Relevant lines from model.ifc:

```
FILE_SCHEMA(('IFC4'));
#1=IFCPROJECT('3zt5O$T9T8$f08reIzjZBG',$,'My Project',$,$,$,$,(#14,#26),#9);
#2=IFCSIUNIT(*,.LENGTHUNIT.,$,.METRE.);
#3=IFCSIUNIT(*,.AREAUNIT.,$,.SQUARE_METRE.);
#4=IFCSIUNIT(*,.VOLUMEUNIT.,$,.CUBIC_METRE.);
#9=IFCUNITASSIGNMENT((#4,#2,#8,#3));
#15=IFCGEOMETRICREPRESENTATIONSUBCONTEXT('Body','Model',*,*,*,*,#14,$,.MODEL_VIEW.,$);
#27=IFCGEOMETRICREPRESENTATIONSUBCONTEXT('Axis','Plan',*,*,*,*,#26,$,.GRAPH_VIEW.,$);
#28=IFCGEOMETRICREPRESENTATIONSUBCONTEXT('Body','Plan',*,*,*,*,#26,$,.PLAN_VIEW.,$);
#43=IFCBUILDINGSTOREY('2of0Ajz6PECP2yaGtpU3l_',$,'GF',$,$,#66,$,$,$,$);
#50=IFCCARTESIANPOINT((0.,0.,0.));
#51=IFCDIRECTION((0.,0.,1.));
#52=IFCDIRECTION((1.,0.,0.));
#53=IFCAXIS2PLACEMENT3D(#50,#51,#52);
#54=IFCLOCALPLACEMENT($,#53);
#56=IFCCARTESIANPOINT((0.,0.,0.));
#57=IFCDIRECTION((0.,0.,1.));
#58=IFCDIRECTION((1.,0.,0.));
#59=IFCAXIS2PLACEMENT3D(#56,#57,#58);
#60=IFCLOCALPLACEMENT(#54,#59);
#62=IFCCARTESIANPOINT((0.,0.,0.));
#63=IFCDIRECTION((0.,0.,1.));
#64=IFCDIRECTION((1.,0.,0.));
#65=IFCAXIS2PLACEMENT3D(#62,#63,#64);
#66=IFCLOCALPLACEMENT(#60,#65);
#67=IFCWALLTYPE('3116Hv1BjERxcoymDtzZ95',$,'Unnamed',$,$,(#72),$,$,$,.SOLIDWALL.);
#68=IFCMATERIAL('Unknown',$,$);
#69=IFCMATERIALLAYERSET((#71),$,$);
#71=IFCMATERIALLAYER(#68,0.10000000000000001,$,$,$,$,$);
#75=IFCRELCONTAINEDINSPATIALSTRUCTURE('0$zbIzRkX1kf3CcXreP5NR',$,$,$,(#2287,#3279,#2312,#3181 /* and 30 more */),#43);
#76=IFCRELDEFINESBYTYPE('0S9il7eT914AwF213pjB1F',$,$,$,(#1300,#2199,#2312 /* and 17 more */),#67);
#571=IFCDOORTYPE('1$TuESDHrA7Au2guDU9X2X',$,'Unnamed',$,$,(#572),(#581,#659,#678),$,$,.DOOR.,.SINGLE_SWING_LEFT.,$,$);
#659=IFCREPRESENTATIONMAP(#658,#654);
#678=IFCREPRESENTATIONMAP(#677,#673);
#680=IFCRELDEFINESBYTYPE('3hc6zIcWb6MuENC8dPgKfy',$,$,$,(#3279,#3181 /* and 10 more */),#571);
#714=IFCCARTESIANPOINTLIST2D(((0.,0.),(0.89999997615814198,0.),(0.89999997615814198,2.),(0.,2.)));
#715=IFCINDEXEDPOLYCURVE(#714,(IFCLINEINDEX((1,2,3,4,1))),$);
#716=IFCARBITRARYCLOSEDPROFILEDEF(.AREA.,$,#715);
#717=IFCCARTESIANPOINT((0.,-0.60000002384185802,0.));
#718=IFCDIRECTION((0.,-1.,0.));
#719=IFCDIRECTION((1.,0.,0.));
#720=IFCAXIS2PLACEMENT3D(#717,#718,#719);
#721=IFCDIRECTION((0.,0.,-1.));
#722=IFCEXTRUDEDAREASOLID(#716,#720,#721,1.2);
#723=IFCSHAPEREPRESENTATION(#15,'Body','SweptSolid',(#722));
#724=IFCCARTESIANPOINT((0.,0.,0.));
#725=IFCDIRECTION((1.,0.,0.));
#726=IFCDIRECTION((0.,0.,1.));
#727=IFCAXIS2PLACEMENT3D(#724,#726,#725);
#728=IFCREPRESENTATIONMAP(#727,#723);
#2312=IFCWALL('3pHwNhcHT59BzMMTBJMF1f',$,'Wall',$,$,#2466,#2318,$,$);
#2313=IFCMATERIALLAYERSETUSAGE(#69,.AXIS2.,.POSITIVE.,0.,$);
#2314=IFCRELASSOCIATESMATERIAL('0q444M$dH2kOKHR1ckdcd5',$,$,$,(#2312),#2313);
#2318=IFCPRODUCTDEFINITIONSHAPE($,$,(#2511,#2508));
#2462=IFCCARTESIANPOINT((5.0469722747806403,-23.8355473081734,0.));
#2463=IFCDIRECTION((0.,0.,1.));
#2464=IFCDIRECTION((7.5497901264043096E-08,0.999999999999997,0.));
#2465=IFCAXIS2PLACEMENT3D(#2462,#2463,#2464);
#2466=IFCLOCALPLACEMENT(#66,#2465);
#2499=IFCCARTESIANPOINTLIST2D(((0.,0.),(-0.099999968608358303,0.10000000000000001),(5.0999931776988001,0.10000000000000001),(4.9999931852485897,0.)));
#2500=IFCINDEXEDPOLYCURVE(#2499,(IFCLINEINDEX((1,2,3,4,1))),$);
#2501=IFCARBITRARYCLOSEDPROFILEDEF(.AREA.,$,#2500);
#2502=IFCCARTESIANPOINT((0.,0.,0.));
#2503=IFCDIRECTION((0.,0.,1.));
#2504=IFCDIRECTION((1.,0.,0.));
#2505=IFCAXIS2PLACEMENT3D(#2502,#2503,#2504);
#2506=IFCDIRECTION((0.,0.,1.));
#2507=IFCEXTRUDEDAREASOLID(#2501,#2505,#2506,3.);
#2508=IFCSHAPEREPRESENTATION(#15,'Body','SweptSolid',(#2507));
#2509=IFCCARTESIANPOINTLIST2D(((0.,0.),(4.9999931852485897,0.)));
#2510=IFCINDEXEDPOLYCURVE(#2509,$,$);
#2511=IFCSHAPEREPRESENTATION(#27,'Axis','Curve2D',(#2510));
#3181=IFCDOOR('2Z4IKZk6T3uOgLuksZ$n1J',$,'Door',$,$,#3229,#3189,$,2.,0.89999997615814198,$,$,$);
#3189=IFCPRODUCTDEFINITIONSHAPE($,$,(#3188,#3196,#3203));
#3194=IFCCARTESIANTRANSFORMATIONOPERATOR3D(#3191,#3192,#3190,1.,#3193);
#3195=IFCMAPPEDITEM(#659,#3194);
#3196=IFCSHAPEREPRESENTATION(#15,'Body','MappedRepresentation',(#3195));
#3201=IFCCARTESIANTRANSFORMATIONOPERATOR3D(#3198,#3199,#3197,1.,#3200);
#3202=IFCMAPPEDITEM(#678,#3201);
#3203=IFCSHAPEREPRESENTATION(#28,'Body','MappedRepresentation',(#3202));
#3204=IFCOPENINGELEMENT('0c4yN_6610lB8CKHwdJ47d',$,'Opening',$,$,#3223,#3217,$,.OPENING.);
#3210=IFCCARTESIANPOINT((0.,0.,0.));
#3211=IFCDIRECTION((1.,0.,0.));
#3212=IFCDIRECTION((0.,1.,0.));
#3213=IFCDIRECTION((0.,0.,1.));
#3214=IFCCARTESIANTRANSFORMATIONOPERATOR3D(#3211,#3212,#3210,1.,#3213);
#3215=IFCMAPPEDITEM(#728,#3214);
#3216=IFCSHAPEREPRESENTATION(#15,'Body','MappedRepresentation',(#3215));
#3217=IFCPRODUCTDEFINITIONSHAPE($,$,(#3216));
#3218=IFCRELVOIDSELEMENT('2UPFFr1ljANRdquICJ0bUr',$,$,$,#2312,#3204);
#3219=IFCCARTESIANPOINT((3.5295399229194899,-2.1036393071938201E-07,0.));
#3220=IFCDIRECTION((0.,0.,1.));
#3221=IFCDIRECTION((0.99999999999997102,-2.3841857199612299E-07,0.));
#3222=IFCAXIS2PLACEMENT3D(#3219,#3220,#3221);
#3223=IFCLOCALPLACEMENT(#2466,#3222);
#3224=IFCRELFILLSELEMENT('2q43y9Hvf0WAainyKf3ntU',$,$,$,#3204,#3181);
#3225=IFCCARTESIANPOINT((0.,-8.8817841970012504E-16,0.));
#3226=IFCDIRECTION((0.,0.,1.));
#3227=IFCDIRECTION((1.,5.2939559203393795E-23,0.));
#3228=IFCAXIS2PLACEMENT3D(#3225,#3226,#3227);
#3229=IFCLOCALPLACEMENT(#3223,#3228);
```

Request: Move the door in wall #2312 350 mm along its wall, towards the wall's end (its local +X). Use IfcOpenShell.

```python
import ifcopenshell
import ifcopenshell.api.geometry
import ifcopenshell.util.placement
import ifcopenshell.util.unit

model = ifcopenshell.open("model.ifc")
unit_scale = ifcopenshell.util.unit.calculate_unit_scale(model)

door = model.by_id(3181)
opening = door.FillsVoids[0].RelatingOpeningElement
wall = opening.VoidsElements[0].RelatingBuildingElement

wall_matrix = ifcopenshell.util.placement.get_local_placement(wall.ObjectPlacement)
shift = wall_matrix[:3, 0] * 0.35 / unit_scale
before = ifcopenshell.util.placement.get_local_placement(door.ObjectPlacement)[:3, 3].copy()

# The door is placed relative to its opening, so it follows when the opening moves.
matrix = ifcopenshell.util.placement.get_local_placement(opening.ObjectPlacement)
matrix[:3, 3] += shift
ifcopenshell.api.geometry.edit_object_placement(
    model, product=opening, matrix=matrix, is_si=False, should_transform_children=True
)

after = ifcopenshell.util.placement.get_local_placement(door.ObjectPlacement)[:3, 3]
print("door moved by", (after - before).round(3) + 0.0)

model.write("model_v2.ifc")
```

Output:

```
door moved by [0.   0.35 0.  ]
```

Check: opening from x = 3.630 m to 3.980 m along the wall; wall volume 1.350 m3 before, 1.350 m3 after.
